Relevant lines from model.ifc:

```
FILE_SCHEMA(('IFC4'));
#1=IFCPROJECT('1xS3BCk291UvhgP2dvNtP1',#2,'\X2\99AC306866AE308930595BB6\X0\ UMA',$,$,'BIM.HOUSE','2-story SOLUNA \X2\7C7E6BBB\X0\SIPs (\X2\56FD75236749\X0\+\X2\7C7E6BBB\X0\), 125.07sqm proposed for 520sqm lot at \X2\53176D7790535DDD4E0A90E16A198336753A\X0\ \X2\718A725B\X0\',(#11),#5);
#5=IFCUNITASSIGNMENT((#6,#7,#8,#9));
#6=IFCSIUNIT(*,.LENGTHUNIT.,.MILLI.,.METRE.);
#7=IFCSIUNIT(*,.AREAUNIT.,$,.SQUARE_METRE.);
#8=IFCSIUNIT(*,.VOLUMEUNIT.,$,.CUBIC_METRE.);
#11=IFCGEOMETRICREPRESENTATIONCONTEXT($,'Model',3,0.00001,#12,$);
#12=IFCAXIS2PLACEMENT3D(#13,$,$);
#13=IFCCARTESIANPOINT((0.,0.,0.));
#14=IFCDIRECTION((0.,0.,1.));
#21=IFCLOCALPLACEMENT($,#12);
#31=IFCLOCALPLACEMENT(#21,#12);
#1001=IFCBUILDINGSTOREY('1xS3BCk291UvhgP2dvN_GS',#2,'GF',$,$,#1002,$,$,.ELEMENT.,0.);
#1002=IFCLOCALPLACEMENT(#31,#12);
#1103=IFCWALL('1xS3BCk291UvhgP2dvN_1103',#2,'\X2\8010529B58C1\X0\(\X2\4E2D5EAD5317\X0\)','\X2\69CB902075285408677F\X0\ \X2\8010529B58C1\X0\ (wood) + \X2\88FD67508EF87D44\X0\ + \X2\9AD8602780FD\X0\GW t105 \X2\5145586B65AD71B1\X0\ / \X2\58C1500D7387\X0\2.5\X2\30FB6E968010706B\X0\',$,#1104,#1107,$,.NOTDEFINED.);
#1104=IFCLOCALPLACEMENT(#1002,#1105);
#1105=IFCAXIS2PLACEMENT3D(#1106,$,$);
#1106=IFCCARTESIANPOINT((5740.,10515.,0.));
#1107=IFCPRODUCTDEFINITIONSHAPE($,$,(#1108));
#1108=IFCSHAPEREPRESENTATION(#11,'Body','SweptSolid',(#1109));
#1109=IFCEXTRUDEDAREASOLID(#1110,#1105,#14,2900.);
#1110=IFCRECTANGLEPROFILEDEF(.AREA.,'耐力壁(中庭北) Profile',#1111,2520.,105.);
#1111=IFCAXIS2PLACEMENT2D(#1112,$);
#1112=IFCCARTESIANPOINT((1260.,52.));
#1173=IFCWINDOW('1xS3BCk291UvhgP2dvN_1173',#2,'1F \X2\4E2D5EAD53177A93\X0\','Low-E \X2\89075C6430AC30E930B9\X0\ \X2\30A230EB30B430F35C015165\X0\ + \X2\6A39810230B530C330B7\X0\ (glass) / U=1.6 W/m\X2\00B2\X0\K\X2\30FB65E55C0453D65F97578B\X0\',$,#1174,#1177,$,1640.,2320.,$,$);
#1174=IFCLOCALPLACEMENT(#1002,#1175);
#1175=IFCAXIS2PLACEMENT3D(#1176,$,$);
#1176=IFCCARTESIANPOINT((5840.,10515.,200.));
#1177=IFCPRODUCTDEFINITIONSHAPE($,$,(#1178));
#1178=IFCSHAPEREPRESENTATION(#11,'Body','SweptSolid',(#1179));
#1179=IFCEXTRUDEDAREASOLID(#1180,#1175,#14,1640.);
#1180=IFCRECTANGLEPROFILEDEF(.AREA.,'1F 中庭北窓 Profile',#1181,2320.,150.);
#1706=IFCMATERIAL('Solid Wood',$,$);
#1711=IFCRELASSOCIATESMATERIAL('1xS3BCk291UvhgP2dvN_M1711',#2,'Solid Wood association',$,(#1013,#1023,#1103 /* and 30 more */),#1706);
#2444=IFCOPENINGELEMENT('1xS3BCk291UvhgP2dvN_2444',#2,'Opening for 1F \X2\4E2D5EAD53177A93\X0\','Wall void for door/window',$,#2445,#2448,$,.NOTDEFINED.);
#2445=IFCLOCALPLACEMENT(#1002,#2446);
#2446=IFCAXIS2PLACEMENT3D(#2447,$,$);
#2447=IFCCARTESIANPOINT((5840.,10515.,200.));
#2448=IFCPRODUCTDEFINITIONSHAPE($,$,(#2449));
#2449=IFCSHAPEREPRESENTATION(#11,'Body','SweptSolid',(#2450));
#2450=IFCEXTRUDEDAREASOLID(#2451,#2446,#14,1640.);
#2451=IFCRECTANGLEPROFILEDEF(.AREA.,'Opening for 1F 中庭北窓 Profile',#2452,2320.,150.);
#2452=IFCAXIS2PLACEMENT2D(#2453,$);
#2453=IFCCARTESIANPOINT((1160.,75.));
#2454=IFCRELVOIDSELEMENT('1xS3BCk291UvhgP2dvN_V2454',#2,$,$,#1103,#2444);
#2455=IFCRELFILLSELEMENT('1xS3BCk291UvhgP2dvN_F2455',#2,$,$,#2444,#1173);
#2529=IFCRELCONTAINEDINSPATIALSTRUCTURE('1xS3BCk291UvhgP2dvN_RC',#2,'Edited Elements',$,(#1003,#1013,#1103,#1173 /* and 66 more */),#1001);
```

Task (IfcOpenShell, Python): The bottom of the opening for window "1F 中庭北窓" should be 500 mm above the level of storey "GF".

```python
import numpy as np
import ifcopenshell
import ifcopenshell.api.geometry
import ifcopenshell.geom
import ifcopenshell.util.element
import ifcopenshell.util.placement
import ifcopenshell.util.shape
import ifcopenshell.util.unit

model = ifcopenshell.open("model.ifc")
unit_scale = ifcopenshell.util.unit.calculate_unit_scale(model)

window = model.by_guid("1xS3BCk291UvhgP2dvN_1173")
opening = window.FillsVoids[0].RelatingOpeningElement
storey = ifcopenshell.util.element.get_container(window, ifc_class="IfcBuildingStorey")
level = ifcopenshell.util.placement.get_local_placement(storey.ObjectPlacement)[2, 3]

# The opening's origin need not be at the sill, so measure its lowest point.
shape = ifcopenshell.geom.create_shape(ifcopenshell.geom.settings(), opening)
bottom = ifcopenshell.util.shape.get_shape_bottom_elevation(shape, shape.geometry) / unit_scale
dz = level + 500.0 - bottom

shift = np.array([0.0, 0.0, dz])
# The window is not placed relative to its opening, so move both.
for product in (opening, window):
    matrix = ifcopenshell.util.placement.get_local_placement(product.ObjectPlacement)
    matrix[:3, 3] += shift
    ifcopenshell.api.geometry.edit_object_placement(model, product=product, matrix=matrix, is_si=False)

print(f"moved by {dz * unit_scale:+.3f} m")

model.write("model_updated.ifc")
```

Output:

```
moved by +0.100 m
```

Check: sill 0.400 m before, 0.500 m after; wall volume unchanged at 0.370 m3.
